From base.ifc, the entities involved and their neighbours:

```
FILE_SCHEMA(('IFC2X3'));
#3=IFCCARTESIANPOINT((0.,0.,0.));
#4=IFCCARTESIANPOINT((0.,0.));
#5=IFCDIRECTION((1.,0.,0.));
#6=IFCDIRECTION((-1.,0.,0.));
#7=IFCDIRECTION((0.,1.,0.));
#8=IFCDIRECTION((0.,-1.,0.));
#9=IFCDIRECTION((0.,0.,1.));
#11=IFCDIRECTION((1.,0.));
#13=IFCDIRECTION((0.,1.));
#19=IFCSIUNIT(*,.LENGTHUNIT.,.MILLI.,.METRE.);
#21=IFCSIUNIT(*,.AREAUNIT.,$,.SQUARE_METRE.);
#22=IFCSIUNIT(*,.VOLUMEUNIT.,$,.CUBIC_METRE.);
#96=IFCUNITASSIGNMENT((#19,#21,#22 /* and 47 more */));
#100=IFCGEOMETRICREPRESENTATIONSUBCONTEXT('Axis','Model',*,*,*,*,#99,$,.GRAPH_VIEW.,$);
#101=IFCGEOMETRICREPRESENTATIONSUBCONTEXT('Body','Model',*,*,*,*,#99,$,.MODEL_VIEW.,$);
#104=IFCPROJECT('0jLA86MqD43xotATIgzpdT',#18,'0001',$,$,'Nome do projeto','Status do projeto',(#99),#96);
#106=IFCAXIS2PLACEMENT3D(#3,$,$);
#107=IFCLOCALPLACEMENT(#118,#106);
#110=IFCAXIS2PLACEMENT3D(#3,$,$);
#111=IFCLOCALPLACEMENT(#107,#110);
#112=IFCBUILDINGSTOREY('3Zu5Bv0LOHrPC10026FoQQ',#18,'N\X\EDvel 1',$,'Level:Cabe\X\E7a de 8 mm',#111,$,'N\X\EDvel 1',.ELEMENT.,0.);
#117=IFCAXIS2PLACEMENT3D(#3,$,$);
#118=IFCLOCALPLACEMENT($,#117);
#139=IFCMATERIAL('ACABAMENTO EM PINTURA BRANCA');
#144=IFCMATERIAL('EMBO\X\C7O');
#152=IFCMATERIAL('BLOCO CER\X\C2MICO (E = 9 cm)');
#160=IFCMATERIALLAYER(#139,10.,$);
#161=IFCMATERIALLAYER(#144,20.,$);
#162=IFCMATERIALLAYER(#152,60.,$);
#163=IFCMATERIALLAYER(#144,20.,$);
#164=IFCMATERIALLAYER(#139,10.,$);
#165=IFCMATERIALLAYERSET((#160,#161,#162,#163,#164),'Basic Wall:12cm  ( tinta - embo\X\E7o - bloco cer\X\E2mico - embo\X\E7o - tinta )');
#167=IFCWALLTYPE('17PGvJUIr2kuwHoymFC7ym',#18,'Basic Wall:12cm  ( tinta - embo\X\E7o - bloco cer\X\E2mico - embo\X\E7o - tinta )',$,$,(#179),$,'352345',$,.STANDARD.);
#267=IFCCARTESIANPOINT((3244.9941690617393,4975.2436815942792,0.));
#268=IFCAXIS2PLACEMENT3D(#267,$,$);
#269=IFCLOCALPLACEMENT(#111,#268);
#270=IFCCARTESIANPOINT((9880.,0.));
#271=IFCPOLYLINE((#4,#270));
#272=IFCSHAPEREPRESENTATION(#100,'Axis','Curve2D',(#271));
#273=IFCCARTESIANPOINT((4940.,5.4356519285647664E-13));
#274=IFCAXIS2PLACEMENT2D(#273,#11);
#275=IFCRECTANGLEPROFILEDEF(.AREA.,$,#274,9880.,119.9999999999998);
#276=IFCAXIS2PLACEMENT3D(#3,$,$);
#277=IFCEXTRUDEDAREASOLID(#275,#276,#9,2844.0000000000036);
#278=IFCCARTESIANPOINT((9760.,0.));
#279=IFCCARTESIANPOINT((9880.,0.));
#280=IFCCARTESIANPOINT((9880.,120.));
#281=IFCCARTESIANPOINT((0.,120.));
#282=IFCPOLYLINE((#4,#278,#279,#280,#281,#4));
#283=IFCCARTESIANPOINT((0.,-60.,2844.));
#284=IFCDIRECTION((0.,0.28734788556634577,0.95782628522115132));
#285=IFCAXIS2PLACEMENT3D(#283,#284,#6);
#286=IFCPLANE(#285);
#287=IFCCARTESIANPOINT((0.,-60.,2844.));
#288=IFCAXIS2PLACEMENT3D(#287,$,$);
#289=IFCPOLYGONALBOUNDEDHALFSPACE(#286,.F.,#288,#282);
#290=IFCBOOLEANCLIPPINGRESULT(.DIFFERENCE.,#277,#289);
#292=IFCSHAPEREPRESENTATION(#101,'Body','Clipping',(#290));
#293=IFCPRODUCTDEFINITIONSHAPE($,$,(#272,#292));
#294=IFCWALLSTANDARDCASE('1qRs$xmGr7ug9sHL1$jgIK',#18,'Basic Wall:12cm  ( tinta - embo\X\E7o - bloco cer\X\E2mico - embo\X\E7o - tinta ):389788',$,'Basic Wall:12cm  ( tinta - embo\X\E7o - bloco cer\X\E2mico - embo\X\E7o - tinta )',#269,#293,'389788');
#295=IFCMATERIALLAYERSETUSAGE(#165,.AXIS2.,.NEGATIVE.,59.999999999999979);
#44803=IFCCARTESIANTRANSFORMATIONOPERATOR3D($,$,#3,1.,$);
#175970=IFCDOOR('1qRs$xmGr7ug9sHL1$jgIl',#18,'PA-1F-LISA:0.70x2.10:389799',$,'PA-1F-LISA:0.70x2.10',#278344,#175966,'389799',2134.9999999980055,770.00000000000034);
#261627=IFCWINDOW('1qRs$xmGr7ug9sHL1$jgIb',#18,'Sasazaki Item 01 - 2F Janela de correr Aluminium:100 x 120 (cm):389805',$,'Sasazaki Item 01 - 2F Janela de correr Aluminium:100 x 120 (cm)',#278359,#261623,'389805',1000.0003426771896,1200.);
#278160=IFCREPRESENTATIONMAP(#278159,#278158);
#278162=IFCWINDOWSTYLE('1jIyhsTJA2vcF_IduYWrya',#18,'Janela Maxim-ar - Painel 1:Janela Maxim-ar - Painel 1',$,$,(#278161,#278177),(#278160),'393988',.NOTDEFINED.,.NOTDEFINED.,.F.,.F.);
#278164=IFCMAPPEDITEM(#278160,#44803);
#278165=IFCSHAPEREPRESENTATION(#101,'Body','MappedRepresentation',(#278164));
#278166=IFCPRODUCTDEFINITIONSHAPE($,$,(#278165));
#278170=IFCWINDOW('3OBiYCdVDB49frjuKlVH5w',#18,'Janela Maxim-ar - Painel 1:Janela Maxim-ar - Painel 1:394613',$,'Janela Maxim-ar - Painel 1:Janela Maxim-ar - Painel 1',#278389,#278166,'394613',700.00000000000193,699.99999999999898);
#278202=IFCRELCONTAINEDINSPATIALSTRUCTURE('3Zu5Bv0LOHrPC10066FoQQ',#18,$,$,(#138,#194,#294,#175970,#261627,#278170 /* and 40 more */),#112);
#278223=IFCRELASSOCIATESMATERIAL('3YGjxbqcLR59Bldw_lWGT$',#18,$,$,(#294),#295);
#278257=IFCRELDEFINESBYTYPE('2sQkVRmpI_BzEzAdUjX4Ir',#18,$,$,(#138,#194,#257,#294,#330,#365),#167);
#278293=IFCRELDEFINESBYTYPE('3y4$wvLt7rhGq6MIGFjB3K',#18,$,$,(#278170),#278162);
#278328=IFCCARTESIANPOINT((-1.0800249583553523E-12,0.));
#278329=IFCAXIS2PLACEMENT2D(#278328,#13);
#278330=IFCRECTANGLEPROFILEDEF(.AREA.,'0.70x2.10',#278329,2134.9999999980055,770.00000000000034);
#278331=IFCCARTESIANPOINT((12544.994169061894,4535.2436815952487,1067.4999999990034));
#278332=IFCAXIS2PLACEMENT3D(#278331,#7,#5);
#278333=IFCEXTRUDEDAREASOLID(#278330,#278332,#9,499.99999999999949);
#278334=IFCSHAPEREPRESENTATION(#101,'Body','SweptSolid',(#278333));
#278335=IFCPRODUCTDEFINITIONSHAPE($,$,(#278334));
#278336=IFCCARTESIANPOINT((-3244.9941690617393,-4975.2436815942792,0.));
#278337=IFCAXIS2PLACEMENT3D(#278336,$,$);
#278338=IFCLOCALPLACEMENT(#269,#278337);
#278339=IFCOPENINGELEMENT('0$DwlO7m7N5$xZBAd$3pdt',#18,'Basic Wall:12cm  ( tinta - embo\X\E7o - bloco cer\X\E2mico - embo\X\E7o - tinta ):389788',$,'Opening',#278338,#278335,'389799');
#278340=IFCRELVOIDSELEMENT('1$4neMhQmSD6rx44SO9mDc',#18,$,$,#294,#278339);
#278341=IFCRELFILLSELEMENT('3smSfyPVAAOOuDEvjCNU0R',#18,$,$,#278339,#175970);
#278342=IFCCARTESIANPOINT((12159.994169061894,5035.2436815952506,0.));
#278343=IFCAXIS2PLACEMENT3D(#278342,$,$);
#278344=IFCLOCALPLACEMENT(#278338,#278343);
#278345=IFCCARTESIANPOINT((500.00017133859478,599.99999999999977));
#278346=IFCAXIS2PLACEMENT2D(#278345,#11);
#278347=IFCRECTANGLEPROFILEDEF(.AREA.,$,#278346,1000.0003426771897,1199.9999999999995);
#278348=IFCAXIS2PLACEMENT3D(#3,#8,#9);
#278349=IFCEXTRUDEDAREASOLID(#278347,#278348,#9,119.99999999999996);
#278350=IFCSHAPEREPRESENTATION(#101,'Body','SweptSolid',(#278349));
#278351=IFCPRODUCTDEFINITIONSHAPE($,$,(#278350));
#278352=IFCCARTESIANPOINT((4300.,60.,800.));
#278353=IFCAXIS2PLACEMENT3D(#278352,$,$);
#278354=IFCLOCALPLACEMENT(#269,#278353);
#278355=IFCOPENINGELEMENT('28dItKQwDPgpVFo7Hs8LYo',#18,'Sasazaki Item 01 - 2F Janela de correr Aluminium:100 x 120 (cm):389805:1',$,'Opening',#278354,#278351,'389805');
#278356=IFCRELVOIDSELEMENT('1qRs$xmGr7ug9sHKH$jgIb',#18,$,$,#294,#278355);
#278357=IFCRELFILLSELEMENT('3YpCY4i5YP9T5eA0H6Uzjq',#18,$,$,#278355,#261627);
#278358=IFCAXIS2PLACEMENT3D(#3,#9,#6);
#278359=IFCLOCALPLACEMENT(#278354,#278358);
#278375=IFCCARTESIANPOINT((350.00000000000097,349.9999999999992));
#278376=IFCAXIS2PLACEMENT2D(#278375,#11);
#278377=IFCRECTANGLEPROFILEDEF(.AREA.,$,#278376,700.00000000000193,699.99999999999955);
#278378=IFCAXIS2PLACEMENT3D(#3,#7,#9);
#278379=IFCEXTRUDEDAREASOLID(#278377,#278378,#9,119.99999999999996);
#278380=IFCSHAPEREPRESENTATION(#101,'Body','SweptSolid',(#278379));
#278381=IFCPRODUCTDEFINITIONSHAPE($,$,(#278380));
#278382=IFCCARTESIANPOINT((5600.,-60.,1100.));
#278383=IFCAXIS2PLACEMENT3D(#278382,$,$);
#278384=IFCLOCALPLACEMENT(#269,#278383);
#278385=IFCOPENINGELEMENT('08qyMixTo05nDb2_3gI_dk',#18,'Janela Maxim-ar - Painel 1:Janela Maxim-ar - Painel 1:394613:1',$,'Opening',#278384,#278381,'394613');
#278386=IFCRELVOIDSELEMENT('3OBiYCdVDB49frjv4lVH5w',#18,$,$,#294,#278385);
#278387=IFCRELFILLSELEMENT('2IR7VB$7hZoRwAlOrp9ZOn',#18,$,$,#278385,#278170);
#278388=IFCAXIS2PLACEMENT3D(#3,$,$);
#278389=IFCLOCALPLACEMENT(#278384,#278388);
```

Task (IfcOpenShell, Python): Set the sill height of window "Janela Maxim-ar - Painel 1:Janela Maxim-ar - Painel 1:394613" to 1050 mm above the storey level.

```python
import numpy as np
import ifcopenshell
import ifcopenshell.api.geometry
import ifcopenshell.geom
import ifcopenshell.util.element
import ifcopenshell.util.placement
import ifcopenshell.util.shape
import ifcopenshell.util.unit

model = ifcopenshell.open("base.ifc")
unit_scale = ifcopenshell.util.unit.calculate_unit_scale(model)

window = model.by_guid("3OBiYCdVDB49frjuKlVH5w")
opening = window.FillsVoids[0].RelatingOpeningElement
storey = ifcopenshell.util.element.get_container(window, ifc_class="IfcBuildingStorey")
level = ifcopenshell.util.placement.get_local_placement(storey.ObjectPlacement)[2, 3]

# The opening's origin need not be at the sill, so measure its lowest point.
shape = ifcopenshell.geom.create_shape(ifcopenshell.geom.settings(), opening)
bottom = ifcopenshell.util.shape.get_shape_bottom_elevation(shape, shape.geometry) / unit_scale
dz = level + 1050.0 - bottom

shift = np.array([0.0, 0.0, dz])
# The window is placed relative to its opening, so it follows when the opening moves.
matrix = ifcopenshell.util.placement.get_local_placement(opening.ObjectPlacement)
matrix[:3, 3] += shift
ifcopenshell.api.geometry.edit_object_placement(
    model, product=opening, matrix=matrix, is_si=False, should_transform_children=True
)

print(f"moved by {dz * unit_scale:+.3f} m")

model.write("base_v2.ifc")
```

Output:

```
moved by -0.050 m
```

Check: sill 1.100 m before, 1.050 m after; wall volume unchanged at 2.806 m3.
